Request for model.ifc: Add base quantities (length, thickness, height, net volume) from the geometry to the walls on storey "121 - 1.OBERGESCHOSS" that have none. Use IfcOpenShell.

First a look at what the model holds.

```python
import ifcopenshell
import ifcopenshell.util.element
import ifcopenshell.util.unit

model = ifcopenshell.open("model.ifc")
print(model.schema)
for unit_type in ("LENGTHUNIT", "AREAUNIT", "VOLUMEUNIT"):
    print(unit_type, ifcopenshell.util.unit.calculate_unit_scale(model, unit_type))
storey = next(s for s in model.by_type("IfcBuildingStorey") if s.Name == "121 - 1.OBERGESCHOSS")
walls = [e for e in ifcopenshell.util.element.get_decomposition(storey) if e.is_a("IfcWall")]
for e in sorted(walls, key=lambda e: e.id()):
    print(e.id(), e.is_a(), e.Name, list(ifcopenshell.util.element.get_psets(e, qtos_only=True)), sep=" | ")
```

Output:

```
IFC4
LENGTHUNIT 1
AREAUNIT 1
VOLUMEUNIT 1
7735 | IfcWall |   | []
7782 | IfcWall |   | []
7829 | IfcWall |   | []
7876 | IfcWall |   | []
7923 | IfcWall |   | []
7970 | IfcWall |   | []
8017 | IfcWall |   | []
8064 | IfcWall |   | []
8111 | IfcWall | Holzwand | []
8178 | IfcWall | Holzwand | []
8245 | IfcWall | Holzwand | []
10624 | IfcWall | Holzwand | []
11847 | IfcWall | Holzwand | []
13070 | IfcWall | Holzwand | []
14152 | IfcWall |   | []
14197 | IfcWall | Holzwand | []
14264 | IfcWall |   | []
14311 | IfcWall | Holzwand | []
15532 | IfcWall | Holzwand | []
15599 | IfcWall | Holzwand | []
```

```python
import ifcopenshell
import ifcopenshell.api.pset
import ifcopenshell.geom
import ifcopenshell.util.element
import ifcopenshell.util.shape
import ifcopenshell.util.unit

model = ifcopenshell.open("model.ifc")
unit_scale = ifcopenshell.util.unit.calculate_unit_scale(model)
volume_scale = ifcopenshell.util.unit.calculate_unit_scale(model, "VOLUMEUNIT")
settings = ifcopenshell.geom.settings()

storey = next(s for s in model.by_type("IfcBuildingStorey") if s.Name == "121 - 1.OBERGESCHOSS")
walls = [e for e in ifcopenshell.util.element.get_decomposition(storey) if e.is_a("IfcWall")]

for e in sorted(walls, key=lambda e: e.id()):
    if ifcopenshell.util.element.get_psets(e, qtos_only=True, should_inherit=False):
        continue
    # Geometry comes back in metres, in the element's own axes.
    shape = ifcopenshell.geom.create_shape(settings, e)
    values = {
        "Length": ifcopenshell.util.shape.get_x(shape.geometry) / unit_scale,
        "Width": ifcopenshell.util.shape.get_y(shape.geometry) / unit_scale,
        "Height": ifcopenshell.util.shape.get_z(shape.geometry) / unit_scale,
        "NetVolume": ifcopenshell.util.shape.get_volume(shape.geometry) / volume_scale,
    }
    qto = ifcopenshell.api.pset.add_qto(model, product=e, name="Qto_WallBaseQuantities")
    ifcopenshell.api.pset.edit_qto(model, qto=qto, properties=values)
    print(e.id(), {k: round(v, 3) for k, v in values.items()})

model.write("model_edited.ifc")
```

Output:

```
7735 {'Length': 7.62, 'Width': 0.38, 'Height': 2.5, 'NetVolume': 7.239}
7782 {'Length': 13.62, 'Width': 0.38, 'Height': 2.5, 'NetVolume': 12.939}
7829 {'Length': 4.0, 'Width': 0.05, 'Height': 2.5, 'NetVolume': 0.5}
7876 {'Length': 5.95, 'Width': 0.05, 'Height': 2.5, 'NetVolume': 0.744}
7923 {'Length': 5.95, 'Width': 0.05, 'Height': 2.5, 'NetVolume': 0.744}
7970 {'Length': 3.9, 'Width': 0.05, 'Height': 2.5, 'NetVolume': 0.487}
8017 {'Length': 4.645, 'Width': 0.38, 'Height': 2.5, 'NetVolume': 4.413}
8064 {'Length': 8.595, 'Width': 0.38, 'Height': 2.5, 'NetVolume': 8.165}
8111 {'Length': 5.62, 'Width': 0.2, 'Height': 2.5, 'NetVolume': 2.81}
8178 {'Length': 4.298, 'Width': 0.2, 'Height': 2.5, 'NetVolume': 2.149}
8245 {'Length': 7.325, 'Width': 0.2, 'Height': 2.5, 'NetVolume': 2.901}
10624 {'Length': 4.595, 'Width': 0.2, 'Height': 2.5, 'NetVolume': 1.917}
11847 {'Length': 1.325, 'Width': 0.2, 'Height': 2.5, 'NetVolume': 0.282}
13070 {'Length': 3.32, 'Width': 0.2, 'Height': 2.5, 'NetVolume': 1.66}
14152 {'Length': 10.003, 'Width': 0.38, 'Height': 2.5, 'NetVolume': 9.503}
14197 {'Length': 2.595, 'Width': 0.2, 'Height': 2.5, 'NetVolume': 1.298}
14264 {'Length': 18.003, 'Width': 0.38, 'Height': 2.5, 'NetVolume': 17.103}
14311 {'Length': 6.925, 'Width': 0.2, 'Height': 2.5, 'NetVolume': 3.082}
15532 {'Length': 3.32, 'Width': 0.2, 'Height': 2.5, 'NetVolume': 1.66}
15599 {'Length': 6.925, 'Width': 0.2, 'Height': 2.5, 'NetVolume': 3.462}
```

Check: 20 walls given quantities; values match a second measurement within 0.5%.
